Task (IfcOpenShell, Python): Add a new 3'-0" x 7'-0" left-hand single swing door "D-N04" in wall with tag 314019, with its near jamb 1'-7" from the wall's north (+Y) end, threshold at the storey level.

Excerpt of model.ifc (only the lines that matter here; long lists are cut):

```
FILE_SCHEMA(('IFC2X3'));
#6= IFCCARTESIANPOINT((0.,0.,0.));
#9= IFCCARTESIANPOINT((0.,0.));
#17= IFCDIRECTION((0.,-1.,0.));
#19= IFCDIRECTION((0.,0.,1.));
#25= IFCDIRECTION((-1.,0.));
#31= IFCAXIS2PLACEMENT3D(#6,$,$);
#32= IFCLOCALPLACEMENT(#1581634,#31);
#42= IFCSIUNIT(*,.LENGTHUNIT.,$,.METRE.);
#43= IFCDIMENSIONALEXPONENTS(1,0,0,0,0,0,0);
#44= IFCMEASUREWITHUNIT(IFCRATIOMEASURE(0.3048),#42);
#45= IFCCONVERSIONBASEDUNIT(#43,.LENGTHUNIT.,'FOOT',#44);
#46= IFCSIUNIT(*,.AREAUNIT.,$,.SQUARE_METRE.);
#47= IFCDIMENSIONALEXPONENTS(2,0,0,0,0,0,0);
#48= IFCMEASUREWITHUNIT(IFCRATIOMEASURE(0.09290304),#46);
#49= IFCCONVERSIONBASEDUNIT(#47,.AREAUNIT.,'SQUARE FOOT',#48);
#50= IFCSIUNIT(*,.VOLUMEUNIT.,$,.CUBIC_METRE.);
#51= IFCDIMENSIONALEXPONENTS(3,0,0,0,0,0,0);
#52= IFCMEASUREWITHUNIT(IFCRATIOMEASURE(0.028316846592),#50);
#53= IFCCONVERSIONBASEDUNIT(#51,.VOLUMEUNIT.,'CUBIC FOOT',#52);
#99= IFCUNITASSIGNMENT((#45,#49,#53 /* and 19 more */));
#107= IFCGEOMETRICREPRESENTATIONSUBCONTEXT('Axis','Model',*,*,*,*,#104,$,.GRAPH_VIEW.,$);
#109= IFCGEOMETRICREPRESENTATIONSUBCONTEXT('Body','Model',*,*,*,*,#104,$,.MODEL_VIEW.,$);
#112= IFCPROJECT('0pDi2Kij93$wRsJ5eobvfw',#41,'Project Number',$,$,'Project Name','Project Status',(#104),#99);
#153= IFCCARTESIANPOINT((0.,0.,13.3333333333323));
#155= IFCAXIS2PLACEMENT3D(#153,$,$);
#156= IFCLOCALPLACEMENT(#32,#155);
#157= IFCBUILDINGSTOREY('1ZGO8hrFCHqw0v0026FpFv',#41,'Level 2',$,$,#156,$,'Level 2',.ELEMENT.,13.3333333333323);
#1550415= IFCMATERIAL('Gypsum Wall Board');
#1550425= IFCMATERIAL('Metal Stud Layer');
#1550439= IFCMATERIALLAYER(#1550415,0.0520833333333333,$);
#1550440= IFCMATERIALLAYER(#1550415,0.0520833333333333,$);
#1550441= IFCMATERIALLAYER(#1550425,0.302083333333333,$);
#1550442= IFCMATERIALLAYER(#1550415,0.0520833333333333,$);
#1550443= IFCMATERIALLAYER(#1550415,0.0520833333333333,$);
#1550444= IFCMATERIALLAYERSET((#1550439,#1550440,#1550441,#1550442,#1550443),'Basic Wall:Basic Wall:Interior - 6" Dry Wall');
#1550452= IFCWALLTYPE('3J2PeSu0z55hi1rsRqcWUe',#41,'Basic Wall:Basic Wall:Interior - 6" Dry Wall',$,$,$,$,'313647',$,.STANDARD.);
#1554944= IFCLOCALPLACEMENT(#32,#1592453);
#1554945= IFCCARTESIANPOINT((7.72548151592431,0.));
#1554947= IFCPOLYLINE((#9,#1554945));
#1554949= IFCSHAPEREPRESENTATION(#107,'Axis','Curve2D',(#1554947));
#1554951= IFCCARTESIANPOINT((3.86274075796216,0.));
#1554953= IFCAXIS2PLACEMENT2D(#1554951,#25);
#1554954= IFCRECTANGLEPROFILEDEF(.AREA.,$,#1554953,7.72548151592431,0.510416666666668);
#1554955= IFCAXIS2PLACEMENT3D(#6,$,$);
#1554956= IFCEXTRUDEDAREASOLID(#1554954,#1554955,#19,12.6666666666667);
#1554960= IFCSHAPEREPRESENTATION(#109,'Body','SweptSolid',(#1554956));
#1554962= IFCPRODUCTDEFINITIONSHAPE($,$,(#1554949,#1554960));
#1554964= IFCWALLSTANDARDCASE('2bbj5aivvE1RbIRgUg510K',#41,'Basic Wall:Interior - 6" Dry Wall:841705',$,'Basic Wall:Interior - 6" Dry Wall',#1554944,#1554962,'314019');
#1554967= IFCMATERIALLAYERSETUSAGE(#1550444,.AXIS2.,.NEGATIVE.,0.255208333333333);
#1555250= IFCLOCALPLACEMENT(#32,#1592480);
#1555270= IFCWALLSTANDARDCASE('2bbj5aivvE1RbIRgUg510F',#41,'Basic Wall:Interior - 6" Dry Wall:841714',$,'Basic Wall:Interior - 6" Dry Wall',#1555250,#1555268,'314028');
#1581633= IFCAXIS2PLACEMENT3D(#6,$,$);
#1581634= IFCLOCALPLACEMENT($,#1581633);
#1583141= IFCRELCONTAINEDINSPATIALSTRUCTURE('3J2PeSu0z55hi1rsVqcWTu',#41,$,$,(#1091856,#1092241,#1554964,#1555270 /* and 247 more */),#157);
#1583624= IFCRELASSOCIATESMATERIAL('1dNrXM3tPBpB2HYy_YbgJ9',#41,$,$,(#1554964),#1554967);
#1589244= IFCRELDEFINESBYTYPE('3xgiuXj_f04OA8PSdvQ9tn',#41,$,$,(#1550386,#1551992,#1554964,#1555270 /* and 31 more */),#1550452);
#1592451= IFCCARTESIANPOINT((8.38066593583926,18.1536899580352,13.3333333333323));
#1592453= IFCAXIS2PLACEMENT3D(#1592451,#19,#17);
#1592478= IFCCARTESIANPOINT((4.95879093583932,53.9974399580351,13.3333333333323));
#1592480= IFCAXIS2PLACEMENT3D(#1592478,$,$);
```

```python
import numpy as np
import ifcopenshell
import ifcopenshell.api.feature
import ifcopenshell.api.geometry
import ifcopenshell.api.root
import ifcopenshell.api.spatial
import ifcopenshell.api.type
import ifcopenshell.geom
import ifcopenshell.util.element
import ifcopenshell.util.placement
import ifcopenshell.util.representation
import ifcopenshell.util.shape
import ifcopenshell.util.unit

model = ifcopenshell.open("model.ifc")
unit_scale = ifcopenshell.util.unit.calculate_unit_scale(model)
settings = ifcopenshell.geom.settings()


def volume(element):
    """Net volume in cubic metres, openings subtracted."""
    shape = ifcopenshell.geom.create_shape(settings, element)
    return ifcopenshell.util.shape.get_volume(shape.geometry)


wall = model.by_guid("2bbj5aivvE1RbIRgUg510K")
storey = ifcopenshell.util.element.get_container(wall, ifc_class="IfcBuildingStorey")
context = ifcopenshell.util.representation.get_context(model, "Model", "Body", "MODEL_VIEW")
before = volume(wall)

width, height, from_end, sill = 0.9144, 2.1336, 0.4826, 0.0  # metres

# The wall runs along its own X axis, and the end named is its -X end.
wall_shape = ifcopenshell.geom.create_shape(settings, wall)
x, y, z = ifcopenshell.util.shape.get_vertices(wall_shape.geometry).T
start = x.min() + from_end
face, thickness = float(y.min()), float(y.max() - y.min())
wall_matrix = ifcopenshell.util.placement.get_local_placement(wall.ObjectPlacement)
level = ifcopenshell.util.placement.get_local_placement(storey.ObjectPlacement)[2, 3]


def in_wall(x, y):
    """Placement at x, y metres in the wall's axes, at sill height."""
    matrix = wall_matrix.copy()
    matrix[:, 3] = wall_matrix @ np.array([x / unit_scale, y / unit_scale, 0.0, 1.0])
    matrix[2, 3] = level + sill / unit_scale
    return matrix


# Opening: a box that overshoots both wall faces by 50 mm.
opening = ifcopenshell.api.root.create_entity(model, ifc_class="IfcOpeningElement")
box = ifcopenshell.api.geometry.add_wall_representation(
    model, context=context, length=width, height=height, thickness=thickness + 0.1
)
ifcopenshell.api.geometry.assign_representation(model, product=opening, representation=box)
ifcopenshell.api.geometry.edit_object_placement(model, product=opening, matrix=in_wall(start, face - 0.05), is_si=False)
ifcopenshell.api.feature.add_feature(model, feature=opening, element=wall)

door = ifcopenshell.api.root.create_entity(model, ifc_class="IfcDoor", name="D-N04")
door.OverallWidth, door.OverallHeight = width / unit_scale, height / unit_scale
body = ifcopenshell.api.geometry.add_door_representation(
    model,
    context=context,
    overall_width=door.OverallWidth,
    overall_height=door.OverallHeight,
    operation_type="SINGLE_SWING_LEFT",
    lining_properties={"LiningDepth": thickness / unit_scale, "ThresholdDepth": thickness / unit_scale},
)
ifcopenshell.api.geometry.assign_representation(model, product=door, representation=body)
ifcopenshell.api.spatial.assign_container(model, products=[door], relating_structure=storey)
fills = ifcopenshell.api.feature.add_filling(model, opening=opening, element=door)
fills.OwnerHistory = door.OwnerHistory  # required in IFC2X3

# IFC2X3 keeps the operation on the door style.
style = ifcopenshell.api.root.create_entity(model, ifc_class="IfcDoorStyle", name="D-N04")
style.OperationType, style.ConstructionType = "SINGLE_SWING_LEFT", "NOTDEFINED"
style.ParameterTakesPrecedence = style.Sizeable = False
ifcopenshell.api.type.assign_type(model, related_objects=[door], relating_type=style)

# The lining spans the wall, so the door starts at the wall face.
ifcopenshell.api.geometry.edit_object_placement(model, product=door, matrix=in_wall(start, face), is_si=False)

after = volume(wall)

print(f"wall volume {before:.3f} -> {after:.3f} m3")

model.write("model_edited.ifc")
```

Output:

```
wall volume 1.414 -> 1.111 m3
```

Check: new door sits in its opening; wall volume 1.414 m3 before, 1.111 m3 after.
